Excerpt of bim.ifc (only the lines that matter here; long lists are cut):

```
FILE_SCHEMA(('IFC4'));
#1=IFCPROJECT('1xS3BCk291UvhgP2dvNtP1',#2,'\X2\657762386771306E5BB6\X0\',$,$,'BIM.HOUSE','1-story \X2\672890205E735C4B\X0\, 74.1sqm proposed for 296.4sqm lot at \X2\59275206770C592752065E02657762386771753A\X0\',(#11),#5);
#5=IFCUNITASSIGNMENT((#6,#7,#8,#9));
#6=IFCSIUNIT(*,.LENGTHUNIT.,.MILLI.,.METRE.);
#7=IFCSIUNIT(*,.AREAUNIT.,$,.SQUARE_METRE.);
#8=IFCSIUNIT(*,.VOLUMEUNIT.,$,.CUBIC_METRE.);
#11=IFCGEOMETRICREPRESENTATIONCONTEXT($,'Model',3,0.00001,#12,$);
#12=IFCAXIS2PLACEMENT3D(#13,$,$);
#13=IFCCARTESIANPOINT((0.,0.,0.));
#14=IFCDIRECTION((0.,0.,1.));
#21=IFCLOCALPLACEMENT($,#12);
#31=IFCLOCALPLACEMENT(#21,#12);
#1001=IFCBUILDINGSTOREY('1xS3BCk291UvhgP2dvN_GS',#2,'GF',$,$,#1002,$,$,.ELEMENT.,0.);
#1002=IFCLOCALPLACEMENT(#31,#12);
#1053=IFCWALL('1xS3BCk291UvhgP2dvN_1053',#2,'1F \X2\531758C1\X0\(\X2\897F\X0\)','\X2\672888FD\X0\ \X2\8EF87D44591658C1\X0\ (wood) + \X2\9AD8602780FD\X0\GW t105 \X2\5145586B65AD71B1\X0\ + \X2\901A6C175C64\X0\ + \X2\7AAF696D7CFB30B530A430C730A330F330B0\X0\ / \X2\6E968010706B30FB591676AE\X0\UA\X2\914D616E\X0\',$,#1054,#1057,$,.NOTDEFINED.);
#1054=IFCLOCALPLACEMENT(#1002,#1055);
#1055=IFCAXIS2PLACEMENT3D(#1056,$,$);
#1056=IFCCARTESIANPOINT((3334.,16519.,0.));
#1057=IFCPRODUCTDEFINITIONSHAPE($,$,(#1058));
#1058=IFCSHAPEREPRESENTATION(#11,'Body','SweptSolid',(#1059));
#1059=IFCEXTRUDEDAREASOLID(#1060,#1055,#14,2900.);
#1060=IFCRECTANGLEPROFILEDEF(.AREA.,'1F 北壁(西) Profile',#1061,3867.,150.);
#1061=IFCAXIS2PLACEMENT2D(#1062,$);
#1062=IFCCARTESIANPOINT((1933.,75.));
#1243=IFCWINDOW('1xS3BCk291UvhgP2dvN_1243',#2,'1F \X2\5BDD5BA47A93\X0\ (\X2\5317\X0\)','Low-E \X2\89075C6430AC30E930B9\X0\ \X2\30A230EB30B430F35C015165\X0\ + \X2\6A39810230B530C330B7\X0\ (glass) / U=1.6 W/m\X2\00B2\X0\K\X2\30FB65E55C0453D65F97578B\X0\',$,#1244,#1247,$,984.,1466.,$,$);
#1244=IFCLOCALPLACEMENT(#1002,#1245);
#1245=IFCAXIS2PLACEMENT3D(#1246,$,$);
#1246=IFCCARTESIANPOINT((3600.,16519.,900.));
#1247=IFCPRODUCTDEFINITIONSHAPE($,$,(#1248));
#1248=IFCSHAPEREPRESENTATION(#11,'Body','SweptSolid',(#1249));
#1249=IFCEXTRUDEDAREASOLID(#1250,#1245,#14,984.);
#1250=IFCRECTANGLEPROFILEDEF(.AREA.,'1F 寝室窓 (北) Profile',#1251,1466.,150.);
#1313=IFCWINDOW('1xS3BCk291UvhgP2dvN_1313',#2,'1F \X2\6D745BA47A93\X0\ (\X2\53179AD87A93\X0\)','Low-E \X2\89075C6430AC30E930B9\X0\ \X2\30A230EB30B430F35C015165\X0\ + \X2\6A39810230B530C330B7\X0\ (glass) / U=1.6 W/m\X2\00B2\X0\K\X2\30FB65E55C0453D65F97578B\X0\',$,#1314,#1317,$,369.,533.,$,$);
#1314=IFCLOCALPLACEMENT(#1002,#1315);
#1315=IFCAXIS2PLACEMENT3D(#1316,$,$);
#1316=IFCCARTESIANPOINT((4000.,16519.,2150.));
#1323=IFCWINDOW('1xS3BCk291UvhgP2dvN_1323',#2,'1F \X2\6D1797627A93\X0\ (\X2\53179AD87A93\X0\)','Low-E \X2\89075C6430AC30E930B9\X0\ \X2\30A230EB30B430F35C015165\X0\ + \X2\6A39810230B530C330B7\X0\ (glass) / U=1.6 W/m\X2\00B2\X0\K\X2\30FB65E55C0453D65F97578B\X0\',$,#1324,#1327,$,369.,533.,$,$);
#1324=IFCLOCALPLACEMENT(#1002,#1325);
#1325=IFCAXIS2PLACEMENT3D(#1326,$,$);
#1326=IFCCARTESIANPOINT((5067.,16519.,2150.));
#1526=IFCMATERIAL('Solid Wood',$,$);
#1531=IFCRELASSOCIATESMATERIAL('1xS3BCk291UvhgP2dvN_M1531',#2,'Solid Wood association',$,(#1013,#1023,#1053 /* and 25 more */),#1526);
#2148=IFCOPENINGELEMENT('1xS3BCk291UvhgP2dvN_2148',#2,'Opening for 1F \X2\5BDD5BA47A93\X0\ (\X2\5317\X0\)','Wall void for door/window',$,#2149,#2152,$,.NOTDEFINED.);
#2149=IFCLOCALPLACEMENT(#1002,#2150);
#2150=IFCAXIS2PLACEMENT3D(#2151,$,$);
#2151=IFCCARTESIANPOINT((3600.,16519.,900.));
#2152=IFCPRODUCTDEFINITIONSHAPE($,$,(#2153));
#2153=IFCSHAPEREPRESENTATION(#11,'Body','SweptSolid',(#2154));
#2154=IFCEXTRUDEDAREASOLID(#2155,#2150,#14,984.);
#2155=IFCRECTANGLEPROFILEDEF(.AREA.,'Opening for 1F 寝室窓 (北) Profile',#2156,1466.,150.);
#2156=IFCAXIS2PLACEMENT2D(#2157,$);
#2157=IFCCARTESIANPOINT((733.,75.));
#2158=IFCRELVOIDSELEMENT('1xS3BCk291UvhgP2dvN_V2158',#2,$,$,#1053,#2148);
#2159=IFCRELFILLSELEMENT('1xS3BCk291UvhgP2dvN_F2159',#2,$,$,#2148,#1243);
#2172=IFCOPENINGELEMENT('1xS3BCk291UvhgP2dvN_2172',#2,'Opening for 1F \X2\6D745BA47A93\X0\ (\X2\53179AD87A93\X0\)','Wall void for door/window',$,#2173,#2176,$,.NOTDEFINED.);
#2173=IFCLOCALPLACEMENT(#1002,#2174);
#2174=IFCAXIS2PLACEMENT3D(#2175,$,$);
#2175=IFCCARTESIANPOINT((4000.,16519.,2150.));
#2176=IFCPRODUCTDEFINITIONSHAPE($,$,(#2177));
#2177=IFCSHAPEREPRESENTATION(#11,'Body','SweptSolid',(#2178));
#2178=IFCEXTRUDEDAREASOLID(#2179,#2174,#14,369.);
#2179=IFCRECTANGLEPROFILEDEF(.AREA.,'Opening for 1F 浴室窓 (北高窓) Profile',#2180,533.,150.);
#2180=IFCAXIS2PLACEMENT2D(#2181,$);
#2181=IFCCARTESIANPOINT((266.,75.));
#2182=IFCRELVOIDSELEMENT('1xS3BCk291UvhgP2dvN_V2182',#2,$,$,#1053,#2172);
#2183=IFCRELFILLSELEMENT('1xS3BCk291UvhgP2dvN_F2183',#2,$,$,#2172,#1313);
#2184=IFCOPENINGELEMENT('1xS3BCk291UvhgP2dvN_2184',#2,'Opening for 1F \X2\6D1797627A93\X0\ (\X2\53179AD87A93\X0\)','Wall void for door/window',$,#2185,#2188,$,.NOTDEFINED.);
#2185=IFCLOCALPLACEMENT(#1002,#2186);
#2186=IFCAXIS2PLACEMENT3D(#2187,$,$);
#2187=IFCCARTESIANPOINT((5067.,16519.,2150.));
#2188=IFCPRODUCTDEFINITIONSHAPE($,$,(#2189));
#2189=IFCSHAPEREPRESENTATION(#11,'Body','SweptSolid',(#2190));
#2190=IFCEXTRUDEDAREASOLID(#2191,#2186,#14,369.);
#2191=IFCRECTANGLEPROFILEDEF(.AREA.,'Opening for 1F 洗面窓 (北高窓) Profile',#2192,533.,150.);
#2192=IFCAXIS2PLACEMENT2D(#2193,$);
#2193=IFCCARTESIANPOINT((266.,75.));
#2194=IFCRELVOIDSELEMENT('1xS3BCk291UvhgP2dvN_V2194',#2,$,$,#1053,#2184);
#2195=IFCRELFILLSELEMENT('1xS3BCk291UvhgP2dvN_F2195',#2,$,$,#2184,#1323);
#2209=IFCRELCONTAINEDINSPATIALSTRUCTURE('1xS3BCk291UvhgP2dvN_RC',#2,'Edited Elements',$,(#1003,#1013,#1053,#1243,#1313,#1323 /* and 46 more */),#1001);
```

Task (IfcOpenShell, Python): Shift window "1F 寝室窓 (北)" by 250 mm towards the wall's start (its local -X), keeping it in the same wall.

```python
import ifcopenshell
import ifcopenshell.api.geometry
import ifcopenshell.util.placement
import ifcopenshell.util.unit

model = ifcopenshell.open("bim.ifc")
unit_scale = ifcopenshell.util.unit.calculate_unit_scale(model)

window = model.by_guid("1xS3BCk291UvhgP2dvN_1243")
opening = window.FillsVoids[0].RelatingOpeningElement
wall = opening.VoidsElements[0].RelatingBuildingElement

wall_matrix = ifcopenshell.util.placement.get_local_placement(wall.ObjectPlacement)
shift = wall_matrix[:3, 0] * -0.25 / unit_scale
before = ifcopenshell.util.placement.get_local_placement(window.ObjectPlacement)[:3, 3].copy()

# The window is not placed relative to its opening, so move both.
for product in (opening, window):
    matrix = ifcopenshell.util.placement.get_local_placement(product.ObjectPlacement)
    matrix[:3, 3] += shift
    ifcopenshell.api.geometry.edit_object_placement(model, product=product, matrix=matrix, is_si=False)

after = ifcopenshell.util.placement.get_local_placement(window.ObjectPlacement)[:3, 3]
print("window moved by", (after - before).round(3) + 0.0)

model.write("bim_updated.ifc")
```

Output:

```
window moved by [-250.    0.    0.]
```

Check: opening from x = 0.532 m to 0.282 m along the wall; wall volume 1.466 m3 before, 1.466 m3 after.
